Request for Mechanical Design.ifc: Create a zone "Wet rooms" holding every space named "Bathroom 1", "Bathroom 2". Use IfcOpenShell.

First a look at what the model holds.

```python
import ifcopenshell

model = ifcopenshell.open("Mechanical Design.ifc")
print(model.schema)
seen = {}
for space in model.by_type("IfcSpace"):
    seen[space.LongName] = seen.get(space.LongName, 0) + 1
for name, count in sorted(seen.items(), key=str):
    print(count, "x", name)
print("zones:", [z.Name for z in model.by_type("IfcZone")][:20])
```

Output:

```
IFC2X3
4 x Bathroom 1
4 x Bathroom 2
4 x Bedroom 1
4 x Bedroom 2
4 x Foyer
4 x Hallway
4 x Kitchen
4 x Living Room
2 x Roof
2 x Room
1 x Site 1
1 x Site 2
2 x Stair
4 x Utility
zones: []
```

```python
import ifcopenshell
import ifcopenshell.api.group
import ifcopenshell.api.root

model = ifcopenshell.open("Mechanical Design.ifc")

names = {"Bathroom 1", "Bathroom 2"}
spaces = [s for s in model.by_type("IfcSpace") if s.LongName in names]

zone = ifcopenshell.api.root.create_entity(model, ifc_class="IfcZone", name="Wet rooms")
ifcopenshell.api.group.assign_group(model, products=spaces, group=zone)
print(len(spaces), "spaces in", zone.Name)

model.write("Mechanical Design_updated.ifc")
```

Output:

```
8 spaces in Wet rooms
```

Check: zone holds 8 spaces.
